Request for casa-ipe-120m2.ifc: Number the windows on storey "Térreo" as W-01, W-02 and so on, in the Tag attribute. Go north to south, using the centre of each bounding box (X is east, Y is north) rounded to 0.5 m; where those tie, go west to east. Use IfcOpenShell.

First a look at what the model holds.

```python
import ifcopenshell
import ifcopenshell.util.element
import ifcopenshell.util.placement

model = ifcopenshell.open("casa-ipe-120m2.ifc")
print(model.schema)
storey = next(s for s in model.by_type("IfcBuildingStorey") if s.Name == "Térreo")
windows = [e for e in ifcopenshell.util.element.get_decomposition(storey) if e.is_a("IfcWindow")]
for e in sorted(windows, key=lambda e: e.id()):
    origin = ifcopenshell.util.placement.get_local_placement(e.ObjectPlacement)[:3, 3]
    print(e.id(), e.Tag, e.Name, origin.round(2) + 0.0, sep=" | ")
```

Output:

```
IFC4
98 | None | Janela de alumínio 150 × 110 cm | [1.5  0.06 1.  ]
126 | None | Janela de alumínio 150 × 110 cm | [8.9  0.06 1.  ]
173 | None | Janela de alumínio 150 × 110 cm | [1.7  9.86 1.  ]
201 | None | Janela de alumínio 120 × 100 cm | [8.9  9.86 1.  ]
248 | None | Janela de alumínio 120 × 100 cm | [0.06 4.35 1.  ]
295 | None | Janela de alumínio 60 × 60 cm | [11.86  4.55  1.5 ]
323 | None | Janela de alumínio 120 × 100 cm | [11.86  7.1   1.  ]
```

```python
import ifcopenshell
import ifcopenshell.geom
import ifcopenshell.util.element
import ifcopenshell.util.shape

model = ifcopenshell.open("casa-ipe-120m2.ifc")
settings = ifcopenshell.geom.settings()
settings.set("use-world-coords", True)


def centre(element):
    shape = ifcopenshell.geom.create_shape(settings, element)
    return ifcopenshell.util.shape.get_bbox_centroid(shape.geometry)


storey = next(s for s in model.by_type("IfcBuildingStorey") if s.Name == "Térreo")
windows = [e for e in ifcopenshell.util.element.get_decomposition(storey) if e.is_a("IfcWindow")]

# Insertion points can sit at a corner or the storey origin, so sort by the geometry (in metres).
centres = {e: centre(e) for e in windows}
windows.sort(key=lambda e: (-round(centres[e][1] / 0.5), centres[e][0]))

for i, e in enumerate(windows, start=1):
    number = f"W-{i:02d}"
    e.Tag = number
    print(e.id(), number)

model.write("casa-ipe-120m2_updated.ifc")
```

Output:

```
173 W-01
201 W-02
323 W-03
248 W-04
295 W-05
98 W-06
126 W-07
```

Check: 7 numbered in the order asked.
